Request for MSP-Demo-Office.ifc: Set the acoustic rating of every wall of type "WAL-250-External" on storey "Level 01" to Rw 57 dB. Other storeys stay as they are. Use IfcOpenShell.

First a look at what the model holds.

```python
import ifcopenshell
import ifcopenshell.util.element

model = ifcopenshell.open("MSP-Demo-Office.ifc")
print(model.schema)
storey = next(s for s in model.by_type("IfcBuildingStorey") if s.Name == "Level 01")
walls = [e for e in ifcopenshell.util.element.get_decomposition(storey) if e.is_a("IfcWall")]
seen = {}
for e in walls:
    element_type = ifcopenshell.util.element.get_type(e)
    key = (element_type.Name if element_type != e and element_type else None, ifcopenshell.util.element.get_pset(e, "Pset_WallCommon", "AcousticRating"))
    seen[key] = seen.get(key, 0) + 1
for (name, value), count in sorted(seen.items(), key=str):
    print(count, "x", name, "|", value)
```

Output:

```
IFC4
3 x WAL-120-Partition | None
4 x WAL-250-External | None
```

```python
import ifcopenshell
import ifcopenshell.api.pset
import ifcopenshell.util.element

model = ifcopenshell.open("MSP-Demo-Office.ifc")

storey = next(s for s in model.by_type("IfcBuildingStorey") if s.Name == "Level 01")
walls = [e for e in ifcopenshell.util.element.get_decomposition(storey) if e.is_a("IfcWall")]

count = 0
for e in walls:
    element_type = ifcopenshell.util.element.get_type(e)
    if element_type in (None, e) or element_type.Name != "WAL-250-External":
        continue
    # add_pset returns the element's existing set when there is one.
    pset = ifcopenshell.api.pset.add_pset(model, product=e, name="Pset_WallCommon")
    ifcopenshell.api.pset.edit_pset(model, pset=pset, properties={"AcousticRating": "Rw 57 dB"})
    count += 1

print(count, "walls updated")

model.write("MSP-Demo-Office_updated.ifc")
```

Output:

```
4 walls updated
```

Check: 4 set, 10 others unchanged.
